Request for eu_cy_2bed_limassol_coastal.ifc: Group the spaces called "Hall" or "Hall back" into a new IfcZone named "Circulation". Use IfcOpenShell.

First a look at what the model holds.

```python
import ifcopenshell

model = ifcopenshell.open("eu_cy_2bed_limassol_coastal.ifc")
print(model.schema)
seen = {}
for space in model.by_type("IfcSpace"):
    seen[space.LongName] = seen.get(space.LongName, 0) + 1
for name, count in sorted(seen.items(), key=str):
    print(count, "x", name)
print("zones:", [z.Name for z in model.by_type("IfcZone")][:20])
```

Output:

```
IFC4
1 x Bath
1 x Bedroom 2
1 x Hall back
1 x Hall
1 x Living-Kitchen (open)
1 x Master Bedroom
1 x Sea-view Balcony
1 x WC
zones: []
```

```python
import ifcopenshell
import ifcopenshell.api.group
import ifcopenshell.api.root

model = ifcopenshell.open("eu_cy_2bed_limassol_coastal.ifc")

names = {"Hall", "Hall back"}
spaces = [s for s in model.by_type("IfcSpace") if s.LongName in names]

zone = ifcopenshell.api.root.create_entity(model, ifc_class="IfcZone", name="Circulation")
ifcopenshell.api.group.assign_group(model, products=spaces, group=zone)
print(len(spaces), "spaces in", zone.Name)

model.write("eu_cy_2bed_limassol_coastal-out.ifc")
```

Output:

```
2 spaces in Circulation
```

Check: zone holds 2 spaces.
